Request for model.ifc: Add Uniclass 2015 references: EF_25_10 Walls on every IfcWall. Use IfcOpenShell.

First a look at what the model holds.

```python
import ifcopenshell

model = ifcopenshell.open("model.ifc")
print(model.schema)
print("classifications:", [c.Name for c in model.by_type("IfcClassification")])
for ifc_class in ("IfcDoor", "IfcRoof", "IfcStair", "IfcWall", "IfcWindow"):
    print(ifc_class, len(model.by_type(ifc_class)))
```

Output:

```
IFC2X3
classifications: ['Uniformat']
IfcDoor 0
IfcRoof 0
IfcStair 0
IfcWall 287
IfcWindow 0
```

```python
import ifcopenshell
import ifcopenshell.api.classification

model = ifcopenshell.open("model.ifc")

# IFC2X3 requires Source and Edition and has no link from the project to the system.
system = model.create_entity("IfcClassification", Source="NBS", Edition="2015", Name="Uniclass 2015")

codes = {
    "IfcWall": ("EF_25_10", "Walls"),
}
for ifc_class, (code, name) in codes.items():
    products = model.by_type(ifc_class)
    ifcopenshell.api.classification.add_reference(
        model, products=products, classification=system, identification=code, name=name
    )
    print(code, len(products))

model.write("model-out.ifc")
```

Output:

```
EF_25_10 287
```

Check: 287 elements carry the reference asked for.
